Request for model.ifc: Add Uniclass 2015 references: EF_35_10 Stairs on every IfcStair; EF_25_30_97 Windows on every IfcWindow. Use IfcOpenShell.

First a look at what the model holds.

```python
import ifcopenshell

model = ifcopenshell.open("model.ifc")
print(model.schema)
print("classifications:", [c.Name for c in model.by_type("IfcClassification")])
for ifc_class in ("IfcDoor", "IfcRoof", "IfcStair", "IfcWall", "IfcWindow"):
    print(ifc_class, len(model.by_type(ifc_class)))
```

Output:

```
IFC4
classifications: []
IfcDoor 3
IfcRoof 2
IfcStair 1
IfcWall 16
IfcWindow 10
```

```python
import ifcopenshell
import ifcopenshell.api.classification

model = ifcopenshell.open("model.ifc")

system = ifcopenshell.api.classification.add_classification(model, classification="Uniclass 2015")

codes = {
    "IfcStair": ("EF_35_10", "Stairs"),
    "IfcWindow": ("EF_25_30_97", "Windows"),
}
for ifc_class, (code, name) in codes.items():
    products = model.by_type(ifc_class)
    ifcopenshell.api.classification.add_reference(
        model, products=products, classification=system, identification=code, name=name
    )
    print(code, len(products))

model.write("model-out.ifc")
```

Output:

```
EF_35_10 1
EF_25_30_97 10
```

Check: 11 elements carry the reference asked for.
